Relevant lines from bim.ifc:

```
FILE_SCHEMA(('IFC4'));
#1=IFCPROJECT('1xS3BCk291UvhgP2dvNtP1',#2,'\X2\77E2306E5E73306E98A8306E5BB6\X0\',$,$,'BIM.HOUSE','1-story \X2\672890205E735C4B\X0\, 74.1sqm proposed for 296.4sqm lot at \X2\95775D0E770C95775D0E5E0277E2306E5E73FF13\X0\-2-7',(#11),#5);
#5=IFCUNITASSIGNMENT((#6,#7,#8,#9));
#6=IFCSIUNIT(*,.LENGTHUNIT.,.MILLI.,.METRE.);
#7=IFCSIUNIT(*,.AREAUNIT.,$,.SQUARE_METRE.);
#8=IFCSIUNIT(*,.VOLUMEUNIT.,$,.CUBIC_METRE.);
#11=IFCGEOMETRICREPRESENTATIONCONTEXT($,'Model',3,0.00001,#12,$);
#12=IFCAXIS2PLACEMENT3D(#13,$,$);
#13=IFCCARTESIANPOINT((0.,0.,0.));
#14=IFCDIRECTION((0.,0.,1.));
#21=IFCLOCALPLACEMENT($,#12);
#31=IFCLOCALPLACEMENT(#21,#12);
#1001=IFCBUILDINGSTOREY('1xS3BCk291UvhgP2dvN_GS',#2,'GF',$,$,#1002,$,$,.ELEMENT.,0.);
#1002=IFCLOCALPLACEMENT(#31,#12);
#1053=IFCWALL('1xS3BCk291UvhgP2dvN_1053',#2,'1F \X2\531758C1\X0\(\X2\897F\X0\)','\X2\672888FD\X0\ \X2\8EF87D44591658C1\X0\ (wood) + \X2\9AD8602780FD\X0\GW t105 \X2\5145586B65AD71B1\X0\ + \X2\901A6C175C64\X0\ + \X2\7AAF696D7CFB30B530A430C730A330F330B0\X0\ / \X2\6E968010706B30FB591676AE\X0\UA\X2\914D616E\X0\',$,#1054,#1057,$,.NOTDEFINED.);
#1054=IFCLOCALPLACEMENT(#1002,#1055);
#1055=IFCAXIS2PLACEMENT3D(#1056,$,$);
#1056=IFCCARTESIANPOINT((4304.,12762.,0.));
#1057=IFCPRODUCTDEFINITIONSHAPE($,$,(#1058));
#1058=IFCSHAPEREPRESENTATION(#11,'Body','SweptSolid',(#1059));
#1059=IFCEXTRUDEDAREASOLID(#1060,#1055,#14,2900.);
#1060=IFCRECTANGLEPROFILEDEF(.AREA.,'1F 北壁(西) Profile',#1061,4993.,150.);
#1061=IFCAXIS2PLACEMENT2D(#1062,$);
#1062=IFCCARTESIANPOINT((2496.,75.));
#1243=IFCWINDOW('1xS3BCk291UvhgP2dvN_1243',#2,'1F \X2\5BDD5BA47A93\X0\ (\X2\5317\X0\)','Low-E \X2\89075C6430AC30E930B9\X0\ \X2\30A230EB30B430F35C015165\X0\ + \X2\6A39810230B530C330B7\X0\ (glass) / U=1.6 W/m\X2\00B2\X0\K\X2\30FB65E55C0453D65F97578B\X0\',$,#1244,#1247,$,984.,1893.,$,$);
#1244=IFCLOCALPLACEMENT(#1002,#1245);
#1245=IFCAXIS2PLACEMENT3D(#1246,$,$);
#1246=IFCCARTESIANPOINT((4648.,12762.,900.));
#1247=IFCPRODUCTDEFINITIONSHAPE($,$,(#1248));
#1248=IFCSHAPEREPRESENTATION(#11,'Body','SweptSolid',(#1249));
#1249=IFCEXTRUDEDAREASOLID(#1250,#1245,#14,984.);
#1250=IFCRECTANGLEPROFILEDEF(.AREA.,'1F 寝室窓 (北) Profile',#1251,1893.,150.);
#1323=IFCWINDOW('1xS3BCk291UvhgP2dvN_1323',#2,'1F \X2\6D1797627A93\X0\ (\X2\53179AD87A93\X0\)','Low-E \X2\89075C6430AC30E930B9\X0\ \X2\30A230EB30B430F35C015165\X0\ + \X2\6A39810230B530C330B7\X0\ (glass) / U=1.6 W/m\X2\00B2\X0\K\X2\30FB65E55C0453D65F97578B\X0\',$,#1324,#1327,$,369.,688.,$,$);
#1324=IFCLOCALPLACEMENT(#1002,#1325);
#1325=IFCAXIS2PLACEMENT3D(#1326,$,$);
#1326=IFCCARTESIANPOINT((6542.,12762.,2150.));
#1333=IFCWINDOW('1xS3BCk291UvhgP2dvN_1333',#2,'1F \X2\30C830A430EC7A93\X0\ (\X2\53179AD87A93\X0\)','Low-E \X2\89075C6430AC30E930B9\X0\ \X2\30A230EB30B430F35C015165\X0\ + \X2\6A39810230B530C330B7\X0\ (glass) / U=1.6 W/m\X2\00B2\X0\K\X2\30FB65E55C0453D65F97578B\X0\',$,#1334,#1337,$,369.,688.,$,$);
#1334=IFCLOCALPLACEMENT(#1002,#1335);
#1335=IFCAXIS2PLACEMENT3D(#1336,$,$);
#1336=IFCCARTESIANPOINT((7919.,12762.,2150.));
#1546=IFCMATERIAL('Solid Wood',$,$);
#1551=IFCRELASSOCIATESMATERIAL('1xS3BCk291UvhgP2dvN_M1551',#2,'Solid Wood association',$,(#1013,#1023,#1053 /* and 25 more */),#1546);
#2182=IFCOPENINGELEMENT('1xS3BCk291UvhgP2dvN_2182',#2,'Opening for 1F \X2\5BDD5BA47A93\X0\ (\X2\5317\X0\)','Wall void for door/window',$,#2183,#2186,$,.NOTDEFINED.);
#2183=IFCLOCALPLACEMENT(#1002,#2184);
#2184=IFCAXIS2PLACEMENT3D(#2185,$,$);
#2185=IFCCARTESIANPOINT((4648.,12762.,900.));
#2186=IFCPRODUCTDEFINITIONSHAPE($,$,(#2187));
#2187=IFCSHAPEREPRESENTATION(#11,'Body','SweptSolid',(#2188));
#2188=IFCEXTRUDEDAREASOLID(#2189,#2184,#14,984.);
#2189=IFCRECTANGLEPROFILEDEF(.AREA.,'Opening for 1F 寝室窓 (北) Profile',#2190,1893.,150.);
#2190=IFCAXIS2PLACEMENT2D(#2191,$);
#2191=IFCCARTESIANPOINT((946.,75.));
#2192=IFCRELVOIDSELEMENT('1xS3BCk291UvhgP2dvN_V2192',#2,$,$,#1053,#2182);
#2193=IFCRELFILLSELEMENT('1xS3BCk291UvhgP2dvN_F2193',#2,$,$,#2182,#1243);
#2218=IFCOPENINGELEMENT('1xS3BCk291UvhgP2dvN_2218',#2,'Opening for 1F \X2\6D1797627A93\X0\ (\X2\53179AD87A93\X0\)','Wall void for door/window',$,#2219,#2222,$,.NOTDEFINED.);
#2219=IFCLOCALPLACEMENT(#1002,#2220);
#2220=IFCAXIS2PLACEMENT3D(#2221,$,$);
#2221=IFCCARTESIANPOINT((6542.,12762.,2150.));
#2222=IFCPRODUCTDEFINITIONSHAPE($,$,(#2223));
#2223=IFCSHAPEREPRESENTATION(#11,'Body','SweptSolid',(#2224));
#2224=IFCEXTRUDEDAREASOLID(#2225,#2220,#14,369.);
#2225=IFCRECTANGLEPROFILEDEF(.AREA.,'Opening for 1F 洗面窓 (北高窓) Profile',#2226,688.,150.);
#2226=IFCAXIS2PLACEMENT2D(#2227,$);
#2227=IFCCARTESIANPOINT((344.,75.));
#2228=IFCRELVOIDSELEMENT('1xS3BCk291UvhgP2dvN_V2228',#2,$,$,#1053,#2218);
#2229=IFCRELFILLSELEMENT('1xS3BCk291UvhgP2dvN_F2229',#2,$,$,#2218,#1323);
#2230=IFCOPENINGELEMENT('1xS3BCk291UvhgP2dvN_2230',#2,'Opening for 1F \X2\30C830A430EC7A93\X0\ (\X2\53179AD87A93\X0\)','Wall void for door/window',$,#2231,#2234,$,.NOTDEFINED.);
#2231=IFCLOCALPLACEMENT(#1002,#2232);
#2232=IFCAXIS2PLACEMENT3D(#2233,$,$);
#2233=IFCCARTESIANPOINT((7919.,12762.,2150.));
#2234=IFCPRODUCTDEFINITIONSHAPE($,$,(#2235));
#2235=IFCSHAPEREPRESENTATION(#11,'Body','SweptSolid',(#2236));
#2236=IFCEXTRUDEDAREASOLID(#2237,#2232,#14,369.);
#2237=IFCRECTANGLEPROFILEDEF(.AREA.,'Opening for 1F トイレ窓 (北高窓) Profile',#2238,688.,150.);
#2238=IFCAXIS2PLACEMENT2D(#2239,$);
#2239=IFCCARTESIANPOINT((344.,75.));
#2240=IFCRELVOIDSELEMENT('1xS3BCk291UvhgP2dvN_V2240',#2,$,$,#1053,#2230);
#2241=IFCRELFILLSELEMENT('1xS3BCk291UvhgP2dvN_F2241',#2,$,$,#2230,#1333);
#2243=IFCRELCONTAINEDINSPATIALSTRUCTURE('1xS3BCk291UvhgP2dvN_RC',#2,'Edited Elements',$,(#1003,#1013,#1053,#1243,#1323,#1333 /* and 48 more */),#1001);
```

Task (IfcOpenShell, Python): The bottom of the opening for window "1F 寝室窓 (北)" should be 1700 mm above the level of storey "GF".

```python
import numpy as np
import ifcopenshell
import ifcopenshell.api.geometry
import ifcopenshell.geom
import ifcopenshell.util.element
import ifcopenshell.util.placement
import ifcopenshell.util.shape
import ifcopenshell.util.unit

model = ifcopenshell.open("bim.ifc")
unit_scale = ifcopenshell.util.unit.calculate_unit_scale(model)

window = model.by_guid("1xS3BCk291UvhgP2dvN_1243")
opening = window.FillsVoids[0].RelatingOpeningElement
storey = ifcopenshell.util.element.get_container(window, ifc_class="IfcBuildingStorey")
level = ifcopenshell.util.placement.get_local_placement(storey.ObjectPlacement)[2, 3]

# The opening's origin need not be at the sill, so measure its lowest point.
shape = ifcopenshell.geom.create_shape(ifcopenshell.geom.settings(), opening)
bottom = ifcopenshell.util.shape.get_shape_bottom_elevation(shape, shape.geometry) / unit_scale
dz = level + 1.7 / unit_scale - bottom

shift = np.array([0.0, 0.0, dz])
# The window is not placed relative to its opening, so move both.
for product in (opening, window):
    matrix = ifcopenshell.util.placement.get_local_placement(product.ObjectPlacement)
    matrix[:3, 3] += shift
    ifcopenshell.api.geometry.edit_object_placement(model, product=product, matrix=matrix, is_si=False)

print(f"moved by {dz * unit_scale:+.3f} m")

model.write("bim_v2.ifc")
```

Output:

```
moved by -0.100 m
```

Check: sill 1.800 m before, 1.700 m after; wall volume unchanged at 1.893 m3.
